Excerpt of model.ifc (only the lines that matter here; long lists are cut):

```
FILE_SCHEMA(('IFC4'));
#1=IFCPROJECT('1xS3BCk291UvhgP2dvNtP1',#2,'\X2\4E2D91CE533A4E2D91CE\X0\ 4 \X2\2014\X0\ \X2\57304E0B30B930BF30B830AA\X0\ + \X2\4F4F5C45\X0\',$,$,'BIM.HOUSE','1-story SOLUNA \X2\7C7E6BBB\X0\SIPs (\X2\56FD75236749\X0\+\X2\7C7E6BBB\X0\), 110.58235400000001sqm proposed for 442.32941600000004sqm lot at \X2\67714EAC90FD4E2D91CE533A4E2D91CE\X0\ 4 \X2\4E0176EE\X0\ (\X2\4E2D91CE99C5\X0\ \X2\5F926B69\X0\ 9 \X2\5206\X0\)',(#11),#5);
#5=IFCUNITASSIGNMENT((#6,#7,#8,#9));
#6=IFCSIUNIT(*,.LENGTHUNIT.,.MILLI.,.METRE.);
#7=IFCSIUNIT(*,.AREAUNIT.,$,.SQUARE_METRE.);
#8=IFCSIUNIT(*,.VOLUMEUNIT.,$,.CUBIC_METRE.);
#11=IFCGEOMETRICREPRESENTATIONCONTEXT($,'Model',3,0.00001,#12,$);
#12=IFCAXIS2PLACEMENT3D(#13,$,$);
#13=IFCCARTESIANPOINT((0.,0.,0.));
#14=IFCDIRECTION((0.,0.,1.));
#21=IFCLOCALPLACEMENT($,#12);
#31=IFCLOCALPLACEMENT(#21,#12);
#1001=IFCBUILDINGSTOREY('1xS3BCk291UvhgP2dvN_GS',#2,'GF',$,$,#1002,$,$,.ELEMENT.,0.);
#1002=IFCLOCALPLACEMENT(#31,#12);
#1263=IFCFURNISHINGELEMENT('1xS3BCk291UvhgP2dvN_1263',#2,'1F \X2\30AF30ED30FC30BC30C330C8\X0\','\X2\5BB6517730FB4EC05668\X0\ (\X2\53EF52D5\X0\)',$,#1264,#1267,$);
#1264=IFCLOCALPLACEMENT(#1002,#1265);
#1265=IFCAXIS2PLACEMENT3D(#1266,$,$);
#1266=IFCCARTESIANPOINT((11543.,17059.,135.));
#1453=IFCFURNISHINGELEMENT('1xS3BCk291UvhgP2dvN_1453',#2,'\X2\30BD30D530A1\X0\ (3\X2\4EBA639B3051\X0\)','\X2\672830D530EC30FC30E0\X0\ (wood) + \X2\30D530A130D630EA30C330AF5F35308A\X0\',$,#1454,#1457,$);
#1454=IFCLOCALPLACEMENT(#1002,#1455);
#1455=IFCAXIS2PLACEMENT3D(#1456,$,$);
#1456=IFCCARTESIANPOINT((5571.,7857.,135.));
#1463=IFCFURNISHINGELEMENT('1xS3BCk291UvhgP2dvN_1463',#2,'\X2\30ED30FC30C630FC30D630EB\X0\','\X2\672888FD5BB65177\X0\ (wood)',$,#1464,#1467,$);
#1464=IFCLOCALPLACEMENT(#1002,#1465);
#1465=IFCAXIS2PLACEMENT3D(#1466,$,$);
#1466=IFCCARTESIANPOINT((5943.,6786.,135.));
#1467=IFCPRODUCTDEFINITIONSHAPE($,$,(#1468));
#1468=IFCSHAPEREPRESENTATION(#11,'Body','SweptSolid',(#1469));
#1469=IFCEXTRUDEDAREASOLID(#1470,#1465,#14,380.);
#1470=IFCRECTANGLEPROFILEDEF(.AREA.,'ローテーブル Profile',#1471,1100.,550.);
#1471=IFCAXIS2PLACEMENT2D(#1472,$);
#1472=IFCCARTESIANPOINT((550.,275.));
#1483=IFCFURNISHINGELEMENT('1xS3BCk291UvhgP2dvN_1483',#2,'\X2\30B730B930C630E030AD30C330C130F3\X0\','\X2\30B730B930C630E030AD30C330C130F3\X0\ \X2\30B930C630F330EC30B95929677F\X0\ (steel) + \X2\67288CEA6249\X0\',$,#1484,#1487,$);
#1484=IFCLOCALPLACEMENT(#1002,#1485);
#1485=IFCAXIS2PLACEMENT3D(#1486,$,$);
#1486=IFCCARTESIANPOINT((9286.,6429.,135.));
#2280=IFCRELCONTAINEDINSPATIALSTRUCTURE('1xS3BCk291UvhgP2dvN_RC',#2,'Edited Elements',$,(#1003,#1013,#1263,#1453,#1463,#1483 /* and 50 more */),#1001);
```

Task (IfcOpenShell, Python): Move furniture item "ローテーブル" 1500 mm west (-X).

```python
import ifcopenshell
import ifcopenshell.api.geometry
import ifcopenshell.util.placement
import ifcopenshell.util.unit

model = ifcopenshell.open("model.ifc")
unit_scale = ifcopenshell.util.unit.calculate_unit_scale(model)

item = model.by_id(1463)
matrix = ifcopenshell.util.placement.get_local_placement(item.ObjectPlacement)
matrix[0, 3] -= 1.5 / unit_scale
ifcopenshell.api.geometry.edit_object_placement(model, product=item, matrix=matrix, is_si=False)

print(ifcopenshell.util.placement.get_local_placement(item.ObjectPlacement).round(3) + 0.0)

model.write("model_v2.ifc")
```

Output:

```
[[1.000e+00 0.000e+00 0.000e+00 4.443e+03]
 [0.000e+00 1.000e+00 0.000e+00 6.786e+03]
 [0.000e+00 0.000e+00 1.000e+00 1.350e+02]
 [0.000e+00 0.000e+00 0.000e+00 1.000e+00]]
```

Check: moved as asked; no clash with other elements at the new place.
